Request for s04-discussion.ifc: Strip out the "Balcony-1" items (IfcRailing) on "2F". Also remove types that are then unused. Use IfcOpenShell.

First a look at what the model holds.

```python
import ifcopenshell
import ifcopenshell.util.element

model = ifcopenshell.open("s04-discussion.ifc")
print(model.schema)
storey = next(s for s in model.by_type("IfcBuildingStorey") if s.Name == "2F")
railings = [e for e in ifcopenshell.util.element.get_decomposition(storey) if e.is_a("IfcRailing")]
seen = {}
for e in railings:
    element_type = ifcopenshell.util.element.get_type(e)
    name = element_type.Name if element_type not in (None, e) else None
    seen[name] = seen.get(name, 0) + 1
for name, count in sorted(seen.items(), key=str):
    print(count, "x", name)
```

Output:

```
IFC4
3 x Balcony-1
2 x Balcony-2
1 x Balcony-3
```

```python
import ifcopenshell
import ifcopenshell.api.root
import ifcopenshell.util.element

model = ifcopenshell.open("s04-discussion.ifc")

storey = next(s for s in model.by_type("IfcBuildingStorey") if s.Name == "2F")
railings = [e for e in ifcopenshell.util.element.get_decomposition(storey) if e.is_a("IfcRailing")]
targets = [e for e in railings if (t := ifcopenshell.util.element.get_type(e)) not in (None, e) and t.Name == "Balcony-1"]
types = {ifcopenshell.util.element.get_type(e) for e in targets} - {None, *targets}

for e in targets:
    ifcopenshell.api.root.remove_product(model, product=e)
print(len(targets), "removed")

unused = [t for t in types if not ifcopenshell.util.element.get_types(t)]
for t in unused:
    ifcopenshell.api.root.remove_product(model, product=t)
print(len(unused), "unused types removed")

model.write("s04-discussion_updated.ifc")
```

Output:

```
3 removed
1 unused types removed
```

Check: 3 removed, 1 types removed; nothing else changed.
